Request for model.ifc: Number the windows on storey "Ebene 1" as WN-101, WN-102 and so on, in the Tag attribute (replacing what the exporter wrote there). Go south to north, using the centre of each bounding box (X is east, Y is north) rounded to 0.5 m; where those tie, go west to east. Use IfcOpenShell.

First a look at what the model holds.

```python
import ifcopenshell
import ifcopenshell.util.element
import ifcopenshell.util.placement

model = ifcopenshell.open("model.ifc")
print(model.schema)
storey = next(s for s in model.by_type("IfcBuildingStorey") if s.Name == "Ebene 1")
windows = [e for e in ifcopenshell.util.element.get_decomposition(storey) if e.is_a("IfcWindow")]
for e in sorted(windows, key=lambda e: e.id()):
    origin = ifcopenshell.util.placement.get_local_placement(e.ObjectPlacement)[:3, 3]
    print(e.id(), e.Tag, e.Name, origin.round(2) + 0.0, sep=" | ")
```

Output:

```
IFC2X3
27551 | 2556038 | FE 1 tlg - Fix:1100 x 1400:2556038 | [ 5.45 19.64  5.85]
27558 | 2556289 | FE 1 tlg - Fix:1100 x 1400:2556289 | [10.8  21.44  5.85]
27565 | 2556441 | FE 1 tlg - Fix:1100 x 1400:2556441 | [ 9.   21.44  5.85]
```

```python
import ifcopenshell
import ifcopenshell.geom
import ifcopenshell.util.element
import ifcopenshell.util.shape

model = ifcopenshell.open("model.ifc")
settings = ifcopenshell.geom.settings()
settings.set("use-world-coords", True)


def centre(element):
    shape = ifcopenshell.geom.create_shape(settings, element)
    return ifcopenshell.util.shape.get_bbox_centroid(shape.geometry)


storey = next(s for s in model.by_type("IfcBuildingStorey") if s.Name == "Ebene 1")
windows = [e for e in ifcopenshell.util.element.get_decomposition(storey) if e.is_a("IfcWindow")]

# Insertion points can sit at a corner or the storey origin, so sort by the geometry (in metres).
centres = {e: centre(e) for e in windows}
windows.sort(key=lambda e: (round(centres[e][1] / 0.5), centres[e][0]))

for i, e in enumerate(windows, start=1):
    number = f"WN-1{i:02d}"
    e.Tag = number
    print(e.id(), number)

model.write("model_updated.ifc")
```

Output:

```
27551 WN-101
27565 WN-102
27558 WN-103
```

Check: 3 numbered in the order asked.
